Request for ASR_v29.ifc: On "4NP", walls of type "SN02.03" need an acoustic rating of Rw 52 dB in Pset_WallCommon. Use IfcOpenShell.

First a look at what the model holds.

```python
import ifcopenshell
import ifcopenshell.util.element

model = ifcopenshell.open("ASR_v29.ifc")
print(model.schema)
storey = next(s for s in model.by_type("IfcBuildingStorey") if s.Name == "4NP")
walls = [e for e in ifcopenshell.util.element.get_decomposition(storey) if e.is_a("IfcWall")]
seen = {}
for e in walls:
    element_type = ifcopenshell.util.element.get_type(e)
    key = (element_type.Name if element_type != e and element_type else None, ifcopenshell.util.element.get_pset(e, "Pset_WallCommon", "AcousticRating"))
    seen[key] = seen.get(key, 0) + 1
for (name, value), count in sorted(seen.items(), key=str):
    print(count, "x", name, "|", value)
```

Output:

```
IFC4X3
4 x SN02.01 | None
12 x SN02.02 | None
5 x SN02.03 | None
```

```python
import ifcopenshell
import ifcopenshell.api.pset
import ifcopenshell.util.element

model = ifcopenshell.open("ASR_v29.ifc")

storey = next(s for s in model.by_type("IfcBuildingStorey") if s.Name == "4NP")
walls = [e for e in ifcopenshell.util.element.get_decomposition(storey) if e.is_a("IfcWall")]

count = 0
for e in walls:
    element_type = ifcopenshell.util.element.get_type(e)
    if element_type in (None, e) or element_type.Name != "SN02.03":
        continue
    # add_pset returns the element's existing set when there is one.
    pset = ifcopenshell.api.pset.add_pset(model, product=e, name="Pset_WallCommon")
    ifcopenshell.api.pset.edit_pset(model, pset=pset, properties={"AcousticRating": "Rw 52 dB"})
    count += 1

print(count, "walls updated")

model.write("ASR_v29_rev.ifc")
```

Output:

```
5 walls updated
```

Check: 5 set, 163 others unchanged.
